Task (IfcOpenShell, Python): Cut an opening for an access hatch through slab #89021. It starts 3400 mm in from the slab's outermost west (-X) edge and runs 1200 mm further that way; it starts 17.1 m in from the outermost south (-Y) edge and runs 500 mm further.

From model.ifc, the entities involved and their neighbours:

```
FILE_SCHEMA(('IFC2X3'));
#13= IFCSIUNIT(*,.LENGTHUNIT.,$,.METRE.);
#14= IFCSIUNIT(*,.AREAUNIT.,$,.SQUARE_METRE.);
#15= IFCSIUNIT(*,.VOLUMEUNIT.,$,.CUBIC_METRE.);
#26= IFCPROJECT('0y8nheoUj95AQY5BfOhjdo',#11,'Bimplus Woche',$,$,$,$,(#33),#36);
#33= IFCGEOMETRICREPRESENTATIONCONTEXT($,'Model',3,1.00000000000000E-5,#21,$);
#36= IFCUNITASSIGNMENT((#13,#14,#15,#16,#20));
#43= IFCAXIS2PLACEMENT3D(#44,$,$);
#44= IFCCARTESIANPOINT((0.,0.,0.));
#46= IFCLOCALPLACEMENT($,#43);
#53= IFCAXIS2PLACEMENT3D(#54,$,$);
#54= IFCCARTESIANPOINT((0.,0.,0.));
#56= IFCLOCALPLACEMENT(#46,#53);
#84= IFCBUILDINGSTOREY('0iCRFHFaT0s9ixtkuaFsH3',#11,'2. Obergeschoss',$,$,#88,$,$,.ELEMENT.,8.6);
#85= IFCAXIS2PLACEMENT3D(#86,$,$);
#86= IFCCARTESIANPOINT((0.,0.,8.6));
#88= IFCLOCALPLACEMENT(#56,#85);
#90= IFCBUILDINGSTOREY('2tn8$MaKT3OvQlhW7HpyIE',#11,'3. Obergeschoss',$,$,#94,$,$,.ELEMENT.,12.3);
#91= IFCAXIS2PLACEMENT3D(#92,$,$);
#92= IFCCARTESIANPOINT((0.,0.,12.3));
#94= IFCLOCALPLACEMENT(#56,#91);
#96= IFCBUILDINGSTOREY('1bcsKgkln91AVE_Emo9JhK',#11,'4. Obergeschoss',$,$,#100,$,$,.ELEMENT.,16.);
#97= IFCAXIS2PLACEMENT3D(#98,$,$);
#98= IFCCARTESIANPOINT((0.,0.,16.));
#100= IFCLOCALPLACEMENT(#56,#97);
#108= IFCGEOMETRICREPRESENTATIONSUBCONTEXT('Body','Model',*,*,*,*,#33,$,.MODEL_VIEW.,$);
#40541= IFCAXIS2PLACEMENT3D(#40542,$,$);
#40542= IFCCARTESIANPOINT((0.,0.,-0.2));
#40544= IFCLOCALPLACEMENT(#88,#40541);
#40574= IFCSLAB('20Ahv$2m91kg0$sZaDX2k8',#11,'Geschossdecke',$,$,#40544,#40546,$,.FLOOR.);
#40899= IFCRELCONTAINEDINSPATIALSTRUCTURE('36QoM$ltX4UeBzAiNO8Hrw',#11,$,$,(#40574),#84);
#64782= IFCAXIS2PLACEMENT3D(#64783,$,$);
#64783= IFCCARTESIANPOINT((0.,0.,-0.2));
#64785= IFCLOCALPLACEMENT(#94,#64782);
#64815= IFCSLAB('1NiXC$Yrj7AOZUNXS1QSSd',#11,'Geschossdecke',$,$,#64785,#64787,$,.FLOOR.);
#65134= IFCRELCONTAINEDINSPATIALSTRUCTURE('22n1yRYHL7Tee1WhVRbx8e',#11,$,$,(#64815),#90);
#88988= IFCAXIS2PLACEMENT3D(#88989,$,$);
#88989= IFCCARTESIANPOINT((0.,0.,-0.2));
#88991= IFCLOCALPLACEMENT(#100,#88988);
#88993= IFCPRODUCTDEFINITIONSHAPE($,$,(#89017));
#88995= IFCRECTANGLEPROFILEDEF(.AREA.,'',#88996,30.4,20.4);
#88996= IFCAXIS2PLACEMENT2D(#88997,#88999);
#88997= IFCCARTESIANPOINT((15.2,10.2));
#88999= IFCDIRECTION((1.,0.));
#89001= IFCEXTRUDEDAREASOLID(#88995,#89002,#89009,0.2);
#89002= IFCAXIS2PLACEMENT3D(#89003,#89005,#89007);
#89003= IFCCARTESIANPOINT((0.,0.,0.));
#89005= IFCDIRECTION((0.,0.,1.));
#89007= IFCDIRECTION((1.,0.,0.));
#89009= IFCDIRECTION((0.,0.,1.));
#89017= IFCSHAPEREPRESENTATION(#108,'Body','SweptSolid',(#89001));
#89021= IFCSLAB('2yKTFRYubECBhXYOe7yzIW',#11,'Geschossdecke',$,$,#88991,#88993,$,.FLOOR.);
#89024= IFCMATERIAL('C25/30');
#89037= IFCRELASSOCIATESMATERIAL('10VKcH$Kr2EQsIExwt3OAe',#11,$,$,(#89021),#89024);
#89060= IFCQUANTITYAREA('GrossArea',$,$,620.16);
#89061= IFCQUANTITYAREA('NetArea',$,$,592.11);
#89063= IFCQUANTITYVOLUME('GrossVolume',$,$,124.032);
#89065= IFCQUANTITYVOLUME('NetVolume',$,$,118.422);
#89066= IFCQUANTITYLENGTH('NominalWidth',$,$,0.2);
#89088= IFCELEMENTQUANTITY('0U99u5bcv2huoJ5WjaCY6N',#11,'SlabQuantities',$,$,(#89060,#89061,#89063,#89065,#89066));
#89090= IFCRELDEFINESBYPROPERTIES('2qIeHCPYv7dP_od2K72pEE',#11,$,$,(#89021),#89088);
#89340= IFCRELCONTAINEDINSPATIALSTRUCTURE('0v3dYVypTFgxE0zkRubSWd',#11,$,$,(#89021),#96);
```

```python
import numpy as np
import ifcopenshell
import ifcopenshell.api.feature
import ifcopenshell.api.geometry
import ifcopenshell.api.pset
import ifcopenshell.api.root
import ifcopenshell.geom
import ifcopenshell.util.element
import ifcopenshell.util.placement
import ifcopenshell.util.representation
import ifcopenshell.util.shape
import ifcopenshell.util.unit

model = ifcopenshell.open("model.ifc")
unit_scale = ifcopenshell.util.unit.calculate_unit_scale(model)
area_scale = ifcopenshell.util.unit.calculate_unit_scale(model, "AREAUNIT")
volume_scale = ifcopenshell.util.unit.calculate_unit_scale(model, "VOLUMEUNIT")
settings = ifcopenshell.geom.settings()


def volume(element):
    """Net volume in cubic metres, openings subtracted."""
    shape = ifcopenshell.geom.create_shape(settings, element)
    return ifcopenshell.util.shape.get_volume(shape.geometry)


slab = model.by_guid("2yKTFRYubECBhXYOe7yzIW")
before = volume(slab)

# Extent in the slab's own axes, in metres. The edges named are its -X and -Y sides.
slab_shape = ifcopenshell.geom.create_shape(settings, slab)
vertices = ifcopenshell.util.shape.get_vertices(slab_shape.geometry)
x_min, y_min, bottom = vertices.min(axis=0)
top = vertices[:, 2].max()

opening = ifcopenshell.api.root.create_entity(model, ifc_class="IfcOpeningElement", name="Access hatch opening")
context = ifcopenshell.util.representation.get_context(model, "Model", "Body", "MODEL_VIEW")
width, depth = 1.2, 0.5
outline = [(0.0, 0.0), (width, 0.0), (width, depth), (0.0, depth), (0.0, 0.0)]
# Overshoot both faces by 50 mm so the cut is clean.
shape = ifcopenshell.api.geometry.add_slab_representation(
    model, context=context, depth=top - bottom + 0.1, polyline=outline
)
ifcopenshell.api.geometry.assign_representation(model, product=opening, representation=shape)

matrix = ifcopenshell.util.placement.get_local_placement(slab.ObjectPlacement)
matrix[:, 3] = matrix @ np.append(np.array([x_min + 3.4, y_min + 17.1, bottom - 0.05]) / unit_scale, 1.0)
ifcopenshell.api.geometry.edit_object_placement(model, product=opening, matrix=matrix, is_si=False)
ifcopenshell.api.feature.add_feature(model, feature=opening, element=slab)

after = volume(slab)

# Update the slab's stored quantities.
qto = model.by_id(ifcopenshell.util.element.get_pset(slab, "SlabQuantities", should_inherit=False)["id"])
ifcopenshell.api.pset.edit_qto(model, qto=qto, properties={
    "NetArea": after / (top - bottom) / area_scale,
    "NetVolume": after / volume_scale,
})

print(f"slab volume {before:.3f} -> {after:.3f} m3")

model.write("model-out.ifc")
```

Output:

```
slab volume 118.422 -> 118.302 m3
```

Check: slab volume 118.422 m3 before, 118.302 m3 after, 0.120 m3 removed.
